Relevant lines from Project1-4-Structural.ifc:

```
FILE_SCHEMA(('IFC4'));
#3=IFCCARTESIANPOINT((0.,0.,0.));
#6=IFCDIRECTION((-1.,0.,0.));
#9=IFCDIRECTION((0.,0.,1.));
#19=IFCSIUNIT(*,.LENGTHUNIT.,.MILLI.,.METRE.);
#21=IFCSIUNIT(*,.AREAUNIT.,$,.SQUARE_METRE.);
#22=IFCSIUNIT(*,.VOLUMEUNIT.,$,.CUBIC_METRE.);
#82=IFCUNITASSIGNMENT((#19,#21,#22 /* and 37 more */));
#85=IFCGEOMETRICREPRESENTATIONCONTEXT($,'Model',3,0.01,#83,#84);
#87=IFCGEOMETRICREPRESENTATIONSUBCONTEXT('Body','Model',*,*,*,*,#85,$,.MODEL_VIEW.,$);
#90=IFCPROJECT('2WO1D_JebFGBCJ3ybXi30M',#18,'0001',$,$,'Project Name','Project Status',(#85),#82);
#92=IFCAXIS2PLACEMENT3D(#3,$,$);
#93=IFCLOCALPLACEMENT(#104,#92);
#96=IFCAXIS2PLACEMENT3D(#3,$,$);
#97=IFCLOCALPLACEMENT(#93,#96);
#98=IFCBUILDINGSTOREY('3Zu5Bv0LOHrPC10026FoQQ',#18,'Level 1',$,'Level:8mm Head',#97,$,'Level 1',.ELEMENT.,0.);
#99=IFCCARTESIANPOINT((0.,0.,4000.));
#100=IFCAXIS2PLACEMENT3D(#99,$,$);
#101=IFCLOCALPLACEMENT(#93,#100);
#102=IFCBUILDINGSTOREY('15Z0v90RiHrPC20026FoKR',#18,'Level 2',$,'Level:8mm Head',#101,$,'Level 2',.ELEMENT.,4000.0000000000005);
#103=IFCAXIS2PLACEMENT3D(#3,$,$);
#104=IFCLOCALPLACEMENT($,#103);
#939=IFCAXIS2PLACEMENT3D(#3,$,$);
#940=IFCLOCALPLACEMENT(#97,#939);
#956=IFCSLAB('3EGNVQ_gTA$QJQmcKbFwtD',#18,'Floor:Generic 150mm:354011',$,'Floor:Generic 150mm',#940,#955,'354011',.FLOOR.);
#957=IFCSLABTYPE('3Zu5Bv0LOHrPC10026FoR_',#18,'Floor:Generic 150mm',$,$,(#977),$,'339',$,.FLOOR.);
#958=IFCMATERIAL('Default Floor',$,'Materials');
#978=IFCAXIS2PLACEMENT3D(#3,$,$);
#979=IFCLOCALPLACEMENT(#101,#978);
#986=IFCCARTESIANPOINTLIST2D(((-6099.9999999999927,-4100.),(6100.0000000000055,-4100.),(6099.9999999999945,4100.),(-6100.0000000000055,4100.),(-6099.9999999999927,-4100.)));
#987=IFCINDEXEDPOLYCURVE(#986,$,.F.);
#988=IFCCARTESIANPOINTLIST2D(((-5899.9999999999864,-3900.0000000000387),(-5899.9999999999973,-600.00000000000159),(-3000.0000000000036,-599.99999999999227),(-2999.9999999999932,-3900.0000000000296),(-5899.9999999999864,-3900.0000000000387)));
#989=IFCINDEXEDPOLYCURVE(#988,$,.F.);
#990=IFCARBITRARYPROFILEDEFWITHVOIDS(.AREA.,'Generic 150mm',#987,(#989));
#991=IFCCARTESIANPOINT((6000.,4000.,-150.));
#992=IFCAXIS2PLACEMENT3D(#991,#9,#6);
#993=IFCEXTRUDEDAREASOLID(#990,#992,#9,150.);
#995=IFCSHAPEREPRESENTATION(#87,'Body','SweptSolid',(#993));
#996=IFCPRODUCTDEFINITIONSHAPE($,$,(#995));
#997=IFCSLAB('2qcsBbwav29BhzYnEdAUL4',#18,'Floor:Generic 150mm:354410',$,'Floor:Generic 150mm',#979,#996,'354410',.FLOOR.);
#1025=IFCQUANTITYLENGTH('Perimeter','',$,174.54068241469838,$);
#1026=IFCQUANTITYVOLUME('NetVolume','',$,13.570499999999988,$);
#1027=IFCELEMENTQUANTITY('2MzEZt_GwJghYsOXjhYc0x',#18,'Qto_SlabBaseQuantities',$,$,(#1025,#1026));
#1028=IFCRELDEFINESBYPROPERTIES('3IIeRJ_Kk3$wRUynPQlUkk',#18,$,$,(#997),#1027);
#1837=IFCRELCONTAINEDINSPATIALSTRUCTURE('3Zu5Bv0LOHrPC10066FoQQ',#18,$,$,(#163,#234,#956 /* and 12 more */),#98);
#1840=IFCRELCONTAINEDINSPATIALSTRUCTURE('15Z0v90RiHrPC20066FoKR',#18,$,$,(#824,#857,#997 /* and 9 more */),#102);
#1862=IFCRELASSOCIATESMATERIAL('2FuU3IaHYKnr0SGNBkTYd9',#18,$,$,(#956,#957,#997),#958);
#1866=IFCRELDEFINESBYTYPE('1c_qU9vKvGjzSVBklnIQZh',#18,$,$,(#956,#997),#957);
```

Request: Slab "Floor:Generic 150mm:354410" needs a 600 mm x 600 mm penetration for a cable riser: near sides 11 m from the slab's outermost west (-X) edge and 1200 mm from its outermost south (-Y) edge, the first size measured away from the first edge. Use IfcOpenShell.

```python
import numpy as np
import ifcopenshell
import ifcopenshell.api.feature
import ifcopenshell.api.geometry
import ifcopenshell.api.pset
import ifcopenshell.api.root
import ifcopenshell.geom
import ifcopenshell.util.element
import ifcopenshell.util.placement
import ifcopenshell.util.representation
import ifcopenshell.util.shape
import ifcopenshell.util.unit

model = ifcopenshell.open("Project1-4-Structural.ifc")
unit_scale = ifcopenshell.util.unit.calculate_unit_scale(model)
volume_scale = ifcopenshell.util.unit.calculate_unit_scale(model, "VOLUMEUNIT")
settings = ifcopenshell.geom.settings()


def volume(element):
    """Net volume in cubic metres, openings subtracted."""
    shape = ifcopenshell.geom.create_shape(settings, element)
    return ifcopenshell.util.shape.get_volume(shape.geometry)


slab = model.by_id(997)
before = volume(slab)

# Extent in the slab's own axes, in metres. The edges named are its -X and -Y sides.
slab_shape = ifcopenshell.geom.create_shape(settings, slab)
vertices = ifcopenshell.util.shape.get_vertices(slab_shape.geometry)
x_min, y_min, bottom = vertices.min(axis=0)
top = vertices[:, 2].max()

opening = ifcopenshell.api.root.create_entity(model, ifc_class="IfcOpeningElement", name="Cable riser opening", predefined_type="OPENING")
context = ifcopenshell.util.representation.get_context(model, "Model", "Body", "MODEL_VIEW")
width, depth = 0.6, 0.6
outline = [(0.0, 0.0), (width, 0.0), (width, depth), (0.0, depth), (0.0, 0.0)]
# Overshoot both faces by 50 mm so the cut is clean.
shape = ifcopenshell.api.geometry.add_slab_representation(
    model, context=context, depth=top - bottom + 0.1, polyline=outline
)
ifcopenshell.api.geometry.assign_representation(model, product=opening, representation=shape)

matrix = ifcopenshell.util.placement.get_local_placement(slab.ObjectPlacement)
matrix[:, 3] = matrix @ np.append(np.array([x_min + 11, y_min + 1.2, bottom - 0.05]) / unit_scale, 1.0)
ifcopenshell.api.geometry.edit_object_placement(model, product=opening, matrix=matrix, is_si=False)
ifcopenshell.api.feature.add_feature(model, feature=opening, element=slab)

after = volume(slab)

# Update the slab's stored quantities.
qto = model.by_id(ifcopenshell.util.element.get_pset(slab, "Qto_SlabBaseQuantities", should_inherit=False)["id"])
ifcopenshell.api.pset.edit_qto(model, qto=qto, properties={"NetVolume": after / volume_scale})

print(f"slab volume {before:.3f} -> {after:.3f} m3")

model.write("Project1-4-Structural_updated.ifc")
```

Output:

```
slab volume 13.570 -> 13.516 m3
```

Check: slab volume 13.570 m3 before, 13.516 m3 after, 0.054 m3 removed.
